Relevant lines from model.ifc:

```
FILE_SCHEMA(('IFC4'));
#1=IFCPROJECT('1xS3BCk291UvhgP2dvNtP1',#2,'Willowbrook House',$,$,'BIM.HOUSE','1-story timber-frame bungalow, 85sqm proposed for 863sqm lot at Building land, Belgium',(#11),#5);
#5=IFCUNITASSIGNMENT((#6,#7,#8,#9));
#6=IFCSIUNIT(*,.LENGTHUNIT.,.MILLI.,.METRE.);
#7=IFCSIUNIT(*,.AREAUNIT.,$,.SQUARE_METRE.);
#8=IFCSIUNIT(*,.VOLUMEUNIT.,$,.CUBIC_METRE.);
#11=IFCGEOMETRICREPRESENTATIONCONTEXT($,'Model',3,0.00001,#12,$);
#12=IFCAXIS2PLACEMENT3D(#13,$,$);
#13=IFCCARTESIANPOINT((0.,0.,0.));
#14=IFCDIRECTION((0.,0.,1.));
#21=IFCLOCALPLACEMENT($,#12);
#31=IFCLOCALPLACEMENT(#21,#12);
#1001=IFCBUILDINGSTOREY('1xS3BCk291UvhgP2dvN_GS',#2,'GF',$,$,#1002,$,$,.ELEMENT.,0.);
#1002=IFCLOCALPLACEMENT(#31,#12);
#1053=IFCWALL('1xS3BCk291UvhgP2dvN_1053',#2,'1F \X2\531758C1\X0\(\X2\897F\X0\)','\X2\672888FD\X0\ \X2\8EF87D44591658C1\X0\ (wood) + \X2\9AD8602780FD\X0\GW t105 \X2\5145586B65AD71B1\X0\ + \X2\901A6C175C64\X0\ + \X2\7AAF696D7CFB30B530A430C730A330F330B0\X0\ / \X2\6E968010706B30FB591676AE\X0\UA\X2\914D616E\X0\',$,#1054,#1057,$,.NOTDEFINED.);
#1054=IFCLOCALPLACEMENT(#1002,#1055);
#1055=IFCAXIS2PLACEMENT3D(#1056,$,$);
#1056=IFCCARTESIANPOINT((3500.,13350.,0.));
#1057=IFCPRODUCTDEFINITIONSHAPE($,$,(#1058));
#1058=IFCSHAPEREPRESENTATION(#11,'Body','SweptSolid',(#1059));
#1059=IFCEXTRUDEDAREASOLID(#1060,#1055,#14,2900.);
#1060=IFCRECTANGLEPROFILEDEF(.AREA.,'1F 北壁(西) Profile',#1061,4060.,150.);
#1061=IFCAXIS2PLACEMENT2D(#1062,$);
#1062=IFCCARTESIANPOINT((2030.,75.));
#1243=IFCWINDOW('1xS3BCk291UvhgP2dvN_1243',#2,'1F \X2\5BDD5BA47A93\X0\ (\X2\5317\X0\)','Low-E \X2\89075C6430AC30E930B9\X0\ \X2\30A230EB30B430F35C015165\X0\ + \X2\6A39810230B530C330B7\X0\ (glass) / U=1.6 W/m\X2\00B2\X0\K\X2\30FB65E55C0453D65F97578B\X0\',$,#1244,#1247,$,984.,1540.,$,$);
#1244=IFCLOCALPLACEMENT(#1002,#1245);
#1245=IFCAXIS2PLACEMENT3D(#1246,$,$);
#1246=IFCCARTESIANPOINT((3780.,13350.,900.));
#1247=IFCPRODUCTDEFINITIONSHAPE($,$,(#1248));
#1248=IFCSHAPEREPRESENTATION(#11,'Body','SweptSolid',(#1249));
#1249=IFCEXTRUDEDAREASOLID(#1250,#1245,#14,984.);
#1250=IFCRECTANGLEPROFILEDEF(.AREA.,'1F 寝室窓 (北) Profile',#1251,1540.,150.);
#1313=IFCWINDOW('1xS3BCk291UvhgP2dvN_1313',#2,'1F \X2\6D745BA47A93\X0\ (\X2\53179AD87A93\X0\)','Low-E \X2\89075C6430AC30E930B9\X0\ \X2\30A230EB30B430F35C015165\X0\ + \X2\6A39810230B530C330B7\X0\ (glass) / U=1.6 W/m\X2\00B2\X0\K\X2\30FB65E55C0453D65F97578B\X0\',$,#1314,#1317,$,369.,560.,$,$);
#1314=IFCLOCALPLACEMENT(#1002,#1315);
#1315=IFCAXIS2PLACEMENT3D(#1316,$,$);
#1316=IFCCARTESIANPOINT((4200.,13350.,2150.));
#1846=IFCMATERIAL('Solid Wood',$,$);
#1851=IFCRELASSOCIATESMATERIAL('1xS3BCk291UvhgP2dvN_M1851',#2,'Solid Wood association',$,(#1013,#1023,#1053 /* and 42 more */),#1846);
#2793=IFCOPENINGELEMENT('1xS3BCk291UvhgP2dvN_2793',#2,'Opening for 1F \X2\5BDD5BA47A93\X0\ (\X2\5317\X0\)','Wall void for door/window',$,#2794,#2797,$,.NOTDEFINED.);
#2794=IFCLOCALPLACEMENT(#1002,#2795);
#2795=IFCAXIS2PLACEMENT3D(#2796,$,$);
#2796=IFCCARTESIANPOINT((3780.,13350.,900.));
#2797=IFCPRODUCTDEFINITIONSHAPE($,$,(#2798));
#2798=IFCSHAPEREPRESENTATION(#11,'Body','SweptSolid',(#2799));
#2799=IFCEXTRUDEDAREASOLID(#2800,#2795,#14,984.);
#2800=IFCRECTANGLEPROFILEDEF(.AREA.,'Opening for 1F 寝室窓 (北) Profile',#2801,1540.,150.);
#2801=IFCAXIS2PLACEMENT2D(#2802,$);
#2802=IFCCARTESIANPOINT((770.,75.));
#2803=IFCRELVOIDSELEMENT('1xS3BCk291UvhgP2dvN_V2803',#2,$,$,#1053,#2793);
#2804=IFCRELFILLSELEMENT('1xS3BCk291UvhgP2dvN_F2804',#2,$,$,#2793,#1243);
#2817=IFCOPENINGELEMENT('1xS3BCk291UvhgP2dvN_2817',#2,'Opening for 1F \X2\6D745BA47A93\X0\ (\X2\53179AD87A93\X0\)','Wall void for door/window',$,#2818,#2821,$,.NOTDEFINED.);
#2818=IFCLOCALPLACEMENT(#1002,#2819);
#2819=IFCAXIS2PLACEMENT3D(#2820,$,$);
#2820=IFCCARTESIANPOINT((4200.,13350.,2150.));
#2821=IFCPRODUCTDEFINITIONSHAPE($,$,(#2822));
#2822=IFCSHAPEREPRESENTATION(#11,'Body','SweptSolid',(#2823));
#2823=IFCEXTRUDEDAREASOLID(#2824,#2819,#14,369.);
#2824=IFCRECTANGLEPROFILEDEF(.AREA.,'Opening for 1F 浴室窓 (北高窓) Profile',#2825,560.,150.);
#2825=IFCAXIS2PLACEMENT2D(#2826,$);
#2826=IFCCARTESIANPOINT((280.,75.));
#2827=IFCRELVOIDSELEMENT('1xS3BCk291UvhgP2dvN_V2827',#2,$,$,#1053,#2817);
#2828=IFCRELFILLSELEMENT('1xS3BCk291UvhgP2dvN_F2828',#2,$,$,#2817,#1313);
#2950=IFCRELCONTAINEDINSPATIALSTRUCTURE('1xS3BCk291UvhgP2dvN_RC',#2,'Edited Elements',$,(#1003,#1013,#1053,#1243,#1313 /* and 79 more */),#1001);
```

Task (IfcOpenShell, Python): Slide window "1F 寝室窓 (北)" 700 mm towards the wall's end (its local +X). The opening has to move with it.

```python
import ifcopenshell
import ifcopenshell.api.geometry
import ifcopenshell.util.placement

model = ifcopenshell.open("model.ifc")

window = model.by_guid("1xS3BCk291UvhgP2dvN_1243")
opening = window.FillsVoids[0].RelatingOpeningElement
wall = opening.VoidsElements[0].RelatingBuildingElement

wall_matrix = ifcopenshell.util.placement.get_local_placement(wall.ObjectPlacement)
shift = wall_matrix[:3, 0] * 700.0
before = ifcopenshell.util.placement.get_local_placement(window.ObjectPlacement)[:3, 3].copy()

# The window is not placed relative to its opening, so move both.
for product in (opening, window):
    matrix = ifcopenshell.util.placement.get_local_placement(product.ObjectPlacement)
    matrix[:3, 3] += shift
    ifcopenshell.api.geometry.edit_object_placement(model, product=product, matrix=matrix, is_si=False)

after = ifcopenshell.util.placement.get_local_placement(window.ObjectPlacement)[:3, 3]
print("window moved by", (after - before).round(3) + 0.0)

model.write("model_updated.ifc")
```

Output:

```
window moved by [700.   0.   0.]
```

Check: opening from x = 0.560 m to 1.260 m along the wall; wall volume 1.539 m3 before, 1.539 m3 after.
